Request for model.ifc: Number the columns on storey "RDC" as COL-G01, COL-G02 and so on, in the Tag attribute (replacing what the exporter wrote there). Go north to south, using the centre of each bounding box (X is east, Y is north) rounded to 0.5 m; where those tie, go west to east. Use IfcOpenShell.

First a look at what the model holds.

```python
import ifcopenshell
import ifcopenshell.util.element
import ifcopenshell.util.placement

model = ifcopenshell.open("model.ifc")
print(model.schema)
storey = next(s for s in model.by_type("IfcBuildingStorey") if s.Name == "RDC")
columns = [e for e in ifcopenshell.util.element.get_decomposition(storey) if e.is_a("IfcColumn")]
for e in sorted(columns, key=lambda e: e.id()):
    origin = ifcopenshell.util.placement.get_local_placement(e.ObjectPlacement)[:3, 3]
    print(e.id(), e.Tag, e.Name, origin.round(2) + 0.0, sep=" | ")
```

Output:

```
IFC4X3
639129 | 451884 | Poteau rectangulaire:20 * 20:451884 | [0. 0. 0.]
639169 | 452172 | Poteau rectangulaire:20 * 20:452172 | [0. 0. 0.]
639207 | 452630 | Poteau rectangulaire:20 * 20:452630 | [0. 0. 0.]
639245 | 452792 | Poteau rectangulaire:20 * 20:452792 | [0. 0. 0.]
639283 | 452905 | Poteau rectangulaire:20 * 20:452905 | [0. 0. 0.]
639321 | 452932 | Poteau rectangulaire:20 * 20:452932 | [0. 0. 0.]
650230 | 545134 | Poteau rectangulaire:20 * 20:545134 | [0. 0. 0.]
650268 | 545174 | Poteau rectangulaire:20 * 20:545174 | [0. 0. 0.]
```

```python
import ifcopenshell
import ifcopenshell.geom
import ifcopenshell.util.element
import ifcopenshell.util.shape

model = ifcopenshell.open("model.ifc")
settings = ifcopenshell.geom.settings()
settings.set("use-world-coords", True)


def centre(element):
    shape = ifcopenshell.geom.create_shape(settings, element)
    return ifcopenshell.util.shape.get_bbox_centroid(shape.geometry)


storey = next(s for s in model.by_type("IfcBuildingStorey") if s.Name == "RDC")
columns = [e for e in ifcopenshell.util.element.get_decomposition(storey) if e.is_a("IfcColumn")]

# Insertion points can sit at a corner or the storey origin, so sort by the geometry (in metres).
centres = {e: centre(e) for e in columns}
columns.sort(key=lambda e: (-round(centres[e][1] / 0.5), centres[e][0]))

for i, e in enumerate(columns, start=1):
    number = f"COL-G{i:02d}"
    e.Tag = number
    print(e.id(), number)

model.write("model_updated.ifc")
```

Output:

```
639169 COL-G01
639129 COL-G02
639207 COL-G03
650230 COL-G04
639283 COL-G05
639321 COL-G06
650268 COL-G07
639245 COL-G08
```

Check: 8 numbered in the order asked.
